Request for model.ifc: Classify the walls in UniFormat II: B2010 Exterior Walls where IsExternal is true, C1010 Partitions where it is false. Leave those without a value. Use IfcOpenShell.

First a look at what the model holds.

```python
import ifcopenshell
import ifcopenshell.util.element

model = ifcopenshell.open("model.ifc")
print(model.schema)
print("classifications:", [c.Name for c in model.by_type("IfcClassification")])
values = [ifcopenshell.util.element.get_pset(e, "Pset_WallCommon", "IsExternal") for e in model.by_type("IfcWall")]
for value in (True, False, None):
    print("IsExternal", value, values.count(value))
```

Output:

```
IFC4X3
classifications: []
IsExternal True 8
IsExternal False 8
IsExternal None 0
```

```python
import ifcopenshell
import ifcopenshell.api.classification
import ifcopenshell.util.element

model = ifcopenshell.open("model.ifc")

system = ifcopenshell.api.classification.add_classification(model, classification="UniFormat II")

walls = model.by_type("IfcWall")
external = {e: ifcopenshell.util.element.get_pset(e, "Pset_WallCommon", "IsExternal") for e in walls}
for flag, code, name in ((True, "B2010", "Exterior Walls"), (False, "C1010", "Partitions")):
    products = [e for e in walls if external[e] is flag]
    ifcopenshell.api.classification.add_reference(
        model, products=products, classification=system, identification=code, name=name
    )
    print(code, len(products))

model.write("model_edited.ifc")
```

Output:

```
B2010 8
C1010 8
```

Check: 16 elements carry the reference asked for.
